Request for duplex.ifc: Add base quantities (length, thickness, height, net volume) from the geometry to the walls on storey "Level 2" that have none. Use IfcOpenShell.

First a look at what the model holds.

```python
import ifcopenshell
import ifcopenshell.util.element
import ifcopenshell.util.unit

model = ifcopenshell.open("duplex.ifc")
print(model.schema)
for unit_type in ("LENGTHUNIT", "AREAUNIT", "VOLUMEUNIT"):
    print(unit_type, ifcopenshell.util.unit.calculate_unit_scale(model, unit_type))
storey = next(s for s in model.by_type("IfcBuildingStorey") if s.Name == "Level 2")
walls = [e for e in ifcopenshell.util.element.get_decomposition(storey) if e.is_a("IfcWall")]
for e in sorted(walls, key=lambda e: e.id()):
    print(e.id(), e.is_a(), e.Name, list(ifcopenshell.util.element.get_psets(e, qtos_only=True)), sep=" | ")
```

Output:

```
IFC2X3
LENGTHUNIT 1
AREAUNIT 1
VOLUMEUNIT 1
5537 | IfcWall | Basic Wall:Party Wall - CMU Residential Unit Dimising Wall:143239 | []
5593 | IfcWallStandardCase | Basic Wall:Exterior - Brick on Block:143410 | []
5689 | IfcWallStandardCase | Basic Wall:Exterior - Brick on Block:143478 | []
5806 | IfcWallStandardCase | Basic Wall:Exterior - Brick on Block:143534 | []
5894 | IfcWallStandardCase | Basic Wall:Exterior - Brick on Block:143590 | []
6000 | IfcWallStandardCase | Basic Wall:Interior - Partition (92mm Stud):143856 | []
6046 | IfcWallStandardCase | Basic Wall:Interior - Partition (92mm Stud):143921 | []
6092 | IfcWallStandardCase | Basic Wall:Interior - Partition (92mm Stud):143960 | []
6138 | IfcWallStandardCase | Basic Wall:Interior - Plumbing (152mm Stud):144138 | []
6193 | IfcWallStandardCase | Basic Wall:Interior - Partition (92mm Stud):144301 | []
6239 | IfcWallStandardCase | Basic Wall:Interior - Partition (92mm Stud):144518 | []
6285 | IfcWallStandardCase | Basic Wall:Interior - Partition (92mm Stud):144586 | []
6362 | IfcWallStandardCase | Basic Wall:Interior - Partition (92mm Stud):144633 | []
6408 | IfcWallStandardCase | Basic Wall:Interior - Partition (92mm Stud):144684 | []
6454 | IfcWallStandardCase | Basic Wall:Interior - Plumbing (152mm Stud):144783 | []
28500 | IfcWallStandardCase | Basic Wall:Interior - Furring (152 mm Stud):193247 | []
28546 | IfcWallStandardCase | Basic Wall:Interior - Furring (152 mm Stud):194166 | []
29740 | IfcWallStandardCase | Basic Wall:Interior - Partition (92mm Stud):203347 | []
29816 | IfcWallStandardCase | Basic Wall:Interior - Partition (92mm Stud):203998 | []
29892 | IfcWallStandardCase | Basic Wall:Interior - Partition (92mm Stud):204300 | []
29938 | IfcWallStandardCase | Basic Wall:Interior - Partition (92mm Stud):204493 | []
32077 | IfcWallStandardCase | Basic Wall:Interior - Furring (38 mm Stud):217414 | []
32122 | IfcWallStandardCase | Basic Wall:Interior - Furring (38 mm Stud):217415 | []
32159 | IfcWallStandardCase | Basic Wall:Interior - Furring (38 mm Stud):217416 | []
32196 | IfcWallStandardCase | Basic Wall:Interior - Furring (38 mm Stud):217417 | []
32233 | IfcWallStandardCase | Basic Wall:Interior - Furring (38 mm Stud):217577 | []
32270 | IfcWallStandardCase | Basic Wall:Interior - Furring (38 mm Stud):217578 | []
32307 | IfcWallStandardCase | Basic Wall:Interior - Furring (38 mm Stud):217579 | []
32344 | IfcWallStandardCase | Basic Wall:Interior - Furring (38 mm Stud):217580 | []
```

```python
import ifcopenshell
import ifcopenshell.api.pset
import ifcopenshell.geom
import ifcopenshell.util.element
import ifcopenshell.util.shape
import ifcopenshell.util.unit

model = ifcopenshell.open("duplex.ifc")
unit_scale = ifcopenshell.util.unit.calculate_unit_scale(model)
volume_scale = ifcopenshell.util.unit.calculate_unit_scale(model, "VOLUMEUNIT")
settings = ifcopenshell.geom.settings()

storey = next(s for s in model.by_type("IfcBuildingStorey") if s.Name == "Level 2")
walls = [e for e in ifcopenshell.util.element.get_decomposition(storey) if e.is_a("IfcWall")]

for e in sorted(walls, key=lambda e: e.id()):
    if ifcopenshell.util.element.get_psets(e, qtos_only=True, should_inherit=False):
        continue
    # Geometry comes back in metres, in the element's own axes.
    shape = ifcopenshell.geom.create_shape(settings, e)
    values = {
        "Length": ifcopenshell.util.shape.get_x(shape.geometry) / unit_scale,
        "Width": ifcopenshell.util.shape.get_y(shape.geometry) / unit_scale,
        "Height": ifcopenshell.util.shape.get_z(shape.geometry) / unit_scale,
        "NetVolume": ifcopenshell.util.shape.get_volume(shape.geometry) / volume_scale,
    }
    qto = ifcopenshell.api.pset.add_qto(model, product=e, name="BaseQuantities")
    ifcopenshell.api.pset.edit_qto(model, qto=qto, properties=values)
    print(e.id(), {k: round(v, 3) for k, v in values.items()})

model.write("duplex_v2.ifc")
```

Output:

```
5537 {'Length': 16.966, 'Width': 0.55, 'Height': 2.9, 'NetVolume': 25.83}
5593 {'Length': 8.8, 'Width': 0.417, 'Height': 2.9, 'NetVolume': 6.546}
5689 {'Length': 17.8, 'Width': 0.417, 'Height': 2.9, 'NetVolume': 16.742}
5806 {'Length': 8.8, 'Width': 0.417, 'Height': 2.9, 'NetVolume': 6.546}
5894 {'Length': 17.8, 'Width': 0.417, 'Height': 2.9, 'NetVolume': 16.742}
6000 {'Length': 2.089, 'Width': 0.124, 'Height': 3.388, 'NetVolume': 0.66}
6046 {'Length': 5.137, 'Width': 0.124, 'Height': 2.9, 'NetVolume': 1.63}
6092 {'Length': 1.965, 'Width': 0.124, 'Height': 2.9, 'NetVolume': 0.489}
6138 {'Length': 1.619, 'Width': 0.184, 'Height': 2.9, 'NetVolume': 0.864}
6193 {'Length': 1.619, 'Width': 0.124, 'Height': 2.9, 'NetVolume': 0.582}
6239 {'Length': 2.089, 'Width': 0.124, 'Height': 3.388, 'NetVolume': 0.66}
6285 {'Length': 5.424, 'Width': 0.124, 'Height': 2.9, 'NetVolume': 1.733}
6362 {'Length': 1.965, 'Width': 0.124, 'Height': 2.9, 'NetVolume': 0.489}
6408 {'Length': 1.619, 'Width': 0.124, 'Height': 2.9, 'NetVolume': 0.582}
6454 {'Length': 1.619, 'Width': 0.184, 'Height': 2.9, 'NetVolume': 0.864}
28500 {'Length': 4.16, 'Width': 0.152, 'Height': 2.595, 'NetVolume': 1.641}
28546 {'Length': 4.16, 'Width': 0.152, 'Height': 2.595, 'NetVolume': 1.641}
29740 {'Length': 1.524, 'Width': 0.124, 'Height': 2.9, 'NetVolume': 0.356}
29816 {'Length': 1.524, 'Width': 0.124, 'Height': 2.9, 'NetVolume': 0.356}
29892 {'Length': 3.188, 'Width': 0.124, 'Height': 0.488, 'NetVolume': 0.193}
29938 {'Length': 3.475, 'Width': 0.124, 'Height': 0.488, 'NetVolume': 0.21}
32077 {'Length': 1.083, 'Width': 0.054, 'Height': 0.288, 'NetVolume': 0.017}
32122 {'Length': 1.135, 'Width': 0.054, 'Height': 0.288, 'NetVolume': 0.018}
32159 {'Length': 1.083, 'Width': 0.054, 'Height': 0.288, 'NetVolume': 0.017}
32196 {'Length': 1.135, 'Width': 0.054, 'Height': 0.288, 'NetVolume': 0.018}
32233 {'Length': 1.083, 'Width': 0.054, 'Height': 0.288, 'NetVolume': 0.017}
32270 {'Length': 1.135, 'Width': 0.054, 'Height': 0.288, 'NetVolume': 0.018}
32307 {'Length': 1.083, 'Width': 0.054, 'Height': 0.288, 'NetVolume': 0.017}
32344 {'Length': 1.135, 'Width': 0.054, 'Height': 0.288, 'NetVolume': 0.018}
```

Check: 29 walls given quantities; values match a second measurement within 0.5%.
